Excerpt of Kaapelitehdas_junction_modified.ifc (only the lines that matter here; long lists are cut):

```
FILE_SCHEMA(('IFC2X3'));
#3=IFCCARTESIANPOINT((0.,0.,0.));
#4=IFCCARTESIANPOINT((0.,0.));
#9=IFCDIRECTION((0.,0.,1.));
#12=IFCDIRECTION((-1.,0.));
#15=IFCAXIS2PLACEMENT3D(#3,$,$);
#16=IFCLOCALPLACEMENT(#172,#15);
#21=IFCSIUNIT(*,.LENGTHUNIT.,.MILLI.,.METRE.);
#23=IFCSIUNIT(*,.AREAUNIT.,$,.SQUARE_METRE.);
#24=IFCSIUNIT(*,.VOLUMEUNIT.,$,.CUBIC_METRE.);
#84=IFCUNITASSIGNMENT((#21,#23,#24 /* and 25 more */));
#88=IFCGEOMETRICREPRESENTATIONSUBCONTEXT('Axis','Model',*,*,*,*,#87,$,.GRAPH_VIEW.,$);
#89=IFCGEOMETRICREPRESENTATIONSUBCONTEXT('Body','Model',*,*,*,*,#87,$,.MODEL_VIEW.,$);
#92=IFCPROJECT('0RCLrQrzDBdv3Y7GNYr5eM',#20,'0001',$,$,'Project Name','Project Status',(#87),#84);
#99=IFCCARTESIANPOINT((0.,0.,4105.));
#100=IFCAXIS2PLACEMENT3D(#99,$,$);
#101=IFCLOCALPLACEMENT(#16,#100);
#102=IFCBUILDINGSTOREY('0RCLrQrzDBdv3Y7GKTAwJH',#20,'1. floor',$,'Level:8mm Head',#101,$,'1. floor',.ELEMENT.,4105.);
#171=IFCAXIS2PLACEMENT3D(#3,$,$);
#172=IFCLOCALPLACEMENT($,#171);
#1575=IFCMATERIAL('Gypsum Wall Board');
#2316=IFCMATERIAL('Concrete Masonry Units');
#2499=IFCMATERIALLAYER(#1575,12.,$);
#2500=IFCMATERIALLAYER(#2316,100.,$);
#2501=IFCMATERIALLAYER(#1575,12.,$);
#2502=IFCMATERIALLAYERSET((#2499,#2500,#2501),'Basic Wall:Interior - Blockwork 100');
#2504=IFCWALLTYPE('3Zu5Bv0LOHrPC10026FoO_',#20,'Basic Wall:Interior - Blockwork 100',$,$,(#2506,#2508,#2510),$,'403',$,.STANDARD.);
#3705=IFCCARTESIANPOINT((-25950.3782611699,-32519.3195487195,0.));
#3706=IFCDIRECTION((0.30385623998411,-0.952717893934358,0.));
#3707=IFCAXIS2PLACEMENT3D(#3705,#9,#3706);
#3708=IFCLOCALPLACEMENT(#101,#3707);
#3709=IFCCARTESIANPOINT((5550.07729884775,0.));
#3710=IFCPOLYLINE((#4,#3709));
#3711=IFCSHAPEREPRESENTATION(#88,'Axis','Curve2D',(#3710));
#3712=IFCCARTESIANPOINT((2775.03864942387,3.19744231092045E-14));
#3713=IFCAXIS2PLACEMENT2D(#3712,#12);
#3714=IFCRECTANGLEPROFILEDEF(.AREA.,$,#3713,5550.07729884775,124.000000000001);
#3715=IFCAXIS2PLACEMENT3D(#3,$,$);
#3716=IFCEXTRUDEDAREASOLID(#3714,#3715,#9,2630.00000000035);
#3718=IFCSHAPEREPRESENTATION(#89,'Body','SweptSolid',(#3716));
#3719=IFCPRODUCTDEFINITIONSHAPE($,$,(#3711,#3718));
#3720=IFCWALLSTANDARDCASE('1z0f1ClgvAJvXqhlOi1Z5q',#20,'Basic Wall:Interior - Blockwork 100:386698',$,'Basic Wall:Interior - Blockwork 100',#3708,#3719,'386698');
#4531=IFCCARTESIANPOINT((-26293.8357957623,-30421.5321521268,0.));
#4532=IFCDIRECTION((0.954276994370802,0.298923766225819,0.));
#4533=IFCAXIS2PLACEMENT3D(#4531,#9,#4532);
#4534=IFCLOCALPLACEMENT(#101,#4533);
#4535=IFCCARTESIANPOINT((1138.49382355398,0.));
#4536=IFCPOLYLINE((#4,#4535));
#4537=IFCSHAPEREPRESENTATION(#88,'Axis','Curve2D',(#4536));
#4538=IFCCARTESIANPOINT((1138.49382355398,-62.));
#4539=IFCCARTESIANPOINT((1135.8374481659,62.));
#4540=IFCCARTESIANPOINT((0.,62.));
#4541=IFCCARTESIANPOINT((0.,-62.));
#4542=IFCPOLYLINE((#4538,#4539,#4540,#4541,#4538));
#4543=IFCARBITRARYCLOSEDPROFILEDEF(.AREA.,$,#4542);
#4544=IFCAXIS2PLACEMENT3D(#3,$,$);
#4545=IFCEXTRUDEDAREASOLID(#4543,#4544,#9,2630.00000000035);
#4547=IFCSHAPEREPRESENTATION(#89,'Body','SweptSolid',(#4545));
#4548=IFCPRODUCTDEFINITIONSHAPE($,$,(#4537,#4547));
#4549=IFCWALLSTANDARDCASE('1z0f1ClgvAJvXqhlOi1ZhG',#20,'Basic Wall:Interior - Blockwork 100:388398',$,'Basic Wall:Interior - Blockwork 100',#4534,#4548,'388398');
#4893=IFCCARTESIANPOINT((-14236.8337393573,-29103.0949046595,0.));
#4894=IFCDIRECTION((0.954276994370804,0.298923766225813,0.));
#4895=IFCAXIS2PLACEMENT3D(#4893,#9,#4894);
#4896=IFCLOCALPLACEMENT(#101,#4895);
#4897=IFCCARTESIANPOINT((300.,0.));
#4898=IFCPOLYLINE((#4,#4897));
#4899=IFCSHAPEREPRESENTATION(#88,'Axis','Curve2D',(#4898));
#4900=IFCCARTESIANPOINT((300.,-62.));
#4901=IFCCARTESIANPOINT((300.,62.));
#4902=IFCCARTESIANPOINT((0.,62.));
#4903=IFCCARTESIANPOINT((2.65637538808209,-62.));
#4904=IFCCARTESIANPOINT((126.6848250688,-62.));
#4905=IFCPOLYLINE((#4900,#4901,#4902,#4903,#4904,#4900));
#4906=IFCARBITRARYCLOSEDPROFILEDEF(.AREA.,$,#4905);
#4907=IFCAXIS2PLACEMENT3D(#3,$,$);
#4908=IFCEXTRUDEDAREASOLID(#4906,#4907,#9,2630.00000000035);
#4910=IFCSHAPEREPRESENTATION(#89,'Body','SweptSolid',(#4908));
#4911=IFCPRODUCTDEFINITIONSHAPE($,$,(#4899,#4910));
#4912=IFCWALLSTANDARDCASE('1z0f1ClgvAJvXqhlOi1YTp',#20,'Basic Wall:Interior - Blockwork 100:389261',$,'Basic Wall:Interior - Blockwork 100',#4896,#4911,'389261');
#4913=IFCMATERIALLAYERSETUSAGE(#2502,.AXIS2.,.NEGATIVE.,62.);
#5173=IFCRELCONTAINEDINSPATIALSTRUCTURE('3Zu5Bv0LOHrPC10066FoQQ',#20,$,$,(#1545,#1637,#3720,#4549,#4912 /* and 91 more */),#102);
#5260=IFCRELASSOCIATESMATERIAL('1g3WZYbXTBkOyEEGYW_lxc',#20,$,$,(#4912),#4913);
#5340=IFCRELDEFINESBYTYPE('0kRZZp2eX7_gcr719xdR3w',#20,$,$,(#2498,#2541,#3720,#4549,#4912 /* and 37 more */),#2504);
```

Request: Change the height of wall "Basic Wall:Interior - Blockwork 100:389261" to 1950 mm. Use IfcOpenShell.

```python
import ifcopenshell
import ifcopenshell.geom
import ifcopenshell.util.representation
import ifcopenshell.util.shape
import ifcopenshell.util.unit

model = ifcopenshell.open("Kaapelitehdas_junction_modified.ifc")
unit_scale = ifcopenshell.util.unit.calculate_unit_scale(model)
settings = ifcopenshell.geom.settings()


def volume(element):
    """Net volume in cubic metres, openings subtracted."""
    shape = ifcopenshell.geom.create_shape(settings, element)
    return ifcopenshell.util.shape.get_volume(shape.geometry)


wall = model.by_guid("1z0f1ClgvAJvXqhlOi1YTp")
before = volume(wall)

body = ifcopenshell.util.representation.get_representation(wall, "Model", "Body")
solid = body.Items[0]
old_height = solid.Depth
solid.Depth = 1.95 / unit_scale
after = volume(wall)

print(f"height {old_height:g} -> {solid.Depth:g}, volume {before:.3f} -> {after:.3f} m3")

model.write("Kaapelitehdas_junction_modified_updated.ifc")
```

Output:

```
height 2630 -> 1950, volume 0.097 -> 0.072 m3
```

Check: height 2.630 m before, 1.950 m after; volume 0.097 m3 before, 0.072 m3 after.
